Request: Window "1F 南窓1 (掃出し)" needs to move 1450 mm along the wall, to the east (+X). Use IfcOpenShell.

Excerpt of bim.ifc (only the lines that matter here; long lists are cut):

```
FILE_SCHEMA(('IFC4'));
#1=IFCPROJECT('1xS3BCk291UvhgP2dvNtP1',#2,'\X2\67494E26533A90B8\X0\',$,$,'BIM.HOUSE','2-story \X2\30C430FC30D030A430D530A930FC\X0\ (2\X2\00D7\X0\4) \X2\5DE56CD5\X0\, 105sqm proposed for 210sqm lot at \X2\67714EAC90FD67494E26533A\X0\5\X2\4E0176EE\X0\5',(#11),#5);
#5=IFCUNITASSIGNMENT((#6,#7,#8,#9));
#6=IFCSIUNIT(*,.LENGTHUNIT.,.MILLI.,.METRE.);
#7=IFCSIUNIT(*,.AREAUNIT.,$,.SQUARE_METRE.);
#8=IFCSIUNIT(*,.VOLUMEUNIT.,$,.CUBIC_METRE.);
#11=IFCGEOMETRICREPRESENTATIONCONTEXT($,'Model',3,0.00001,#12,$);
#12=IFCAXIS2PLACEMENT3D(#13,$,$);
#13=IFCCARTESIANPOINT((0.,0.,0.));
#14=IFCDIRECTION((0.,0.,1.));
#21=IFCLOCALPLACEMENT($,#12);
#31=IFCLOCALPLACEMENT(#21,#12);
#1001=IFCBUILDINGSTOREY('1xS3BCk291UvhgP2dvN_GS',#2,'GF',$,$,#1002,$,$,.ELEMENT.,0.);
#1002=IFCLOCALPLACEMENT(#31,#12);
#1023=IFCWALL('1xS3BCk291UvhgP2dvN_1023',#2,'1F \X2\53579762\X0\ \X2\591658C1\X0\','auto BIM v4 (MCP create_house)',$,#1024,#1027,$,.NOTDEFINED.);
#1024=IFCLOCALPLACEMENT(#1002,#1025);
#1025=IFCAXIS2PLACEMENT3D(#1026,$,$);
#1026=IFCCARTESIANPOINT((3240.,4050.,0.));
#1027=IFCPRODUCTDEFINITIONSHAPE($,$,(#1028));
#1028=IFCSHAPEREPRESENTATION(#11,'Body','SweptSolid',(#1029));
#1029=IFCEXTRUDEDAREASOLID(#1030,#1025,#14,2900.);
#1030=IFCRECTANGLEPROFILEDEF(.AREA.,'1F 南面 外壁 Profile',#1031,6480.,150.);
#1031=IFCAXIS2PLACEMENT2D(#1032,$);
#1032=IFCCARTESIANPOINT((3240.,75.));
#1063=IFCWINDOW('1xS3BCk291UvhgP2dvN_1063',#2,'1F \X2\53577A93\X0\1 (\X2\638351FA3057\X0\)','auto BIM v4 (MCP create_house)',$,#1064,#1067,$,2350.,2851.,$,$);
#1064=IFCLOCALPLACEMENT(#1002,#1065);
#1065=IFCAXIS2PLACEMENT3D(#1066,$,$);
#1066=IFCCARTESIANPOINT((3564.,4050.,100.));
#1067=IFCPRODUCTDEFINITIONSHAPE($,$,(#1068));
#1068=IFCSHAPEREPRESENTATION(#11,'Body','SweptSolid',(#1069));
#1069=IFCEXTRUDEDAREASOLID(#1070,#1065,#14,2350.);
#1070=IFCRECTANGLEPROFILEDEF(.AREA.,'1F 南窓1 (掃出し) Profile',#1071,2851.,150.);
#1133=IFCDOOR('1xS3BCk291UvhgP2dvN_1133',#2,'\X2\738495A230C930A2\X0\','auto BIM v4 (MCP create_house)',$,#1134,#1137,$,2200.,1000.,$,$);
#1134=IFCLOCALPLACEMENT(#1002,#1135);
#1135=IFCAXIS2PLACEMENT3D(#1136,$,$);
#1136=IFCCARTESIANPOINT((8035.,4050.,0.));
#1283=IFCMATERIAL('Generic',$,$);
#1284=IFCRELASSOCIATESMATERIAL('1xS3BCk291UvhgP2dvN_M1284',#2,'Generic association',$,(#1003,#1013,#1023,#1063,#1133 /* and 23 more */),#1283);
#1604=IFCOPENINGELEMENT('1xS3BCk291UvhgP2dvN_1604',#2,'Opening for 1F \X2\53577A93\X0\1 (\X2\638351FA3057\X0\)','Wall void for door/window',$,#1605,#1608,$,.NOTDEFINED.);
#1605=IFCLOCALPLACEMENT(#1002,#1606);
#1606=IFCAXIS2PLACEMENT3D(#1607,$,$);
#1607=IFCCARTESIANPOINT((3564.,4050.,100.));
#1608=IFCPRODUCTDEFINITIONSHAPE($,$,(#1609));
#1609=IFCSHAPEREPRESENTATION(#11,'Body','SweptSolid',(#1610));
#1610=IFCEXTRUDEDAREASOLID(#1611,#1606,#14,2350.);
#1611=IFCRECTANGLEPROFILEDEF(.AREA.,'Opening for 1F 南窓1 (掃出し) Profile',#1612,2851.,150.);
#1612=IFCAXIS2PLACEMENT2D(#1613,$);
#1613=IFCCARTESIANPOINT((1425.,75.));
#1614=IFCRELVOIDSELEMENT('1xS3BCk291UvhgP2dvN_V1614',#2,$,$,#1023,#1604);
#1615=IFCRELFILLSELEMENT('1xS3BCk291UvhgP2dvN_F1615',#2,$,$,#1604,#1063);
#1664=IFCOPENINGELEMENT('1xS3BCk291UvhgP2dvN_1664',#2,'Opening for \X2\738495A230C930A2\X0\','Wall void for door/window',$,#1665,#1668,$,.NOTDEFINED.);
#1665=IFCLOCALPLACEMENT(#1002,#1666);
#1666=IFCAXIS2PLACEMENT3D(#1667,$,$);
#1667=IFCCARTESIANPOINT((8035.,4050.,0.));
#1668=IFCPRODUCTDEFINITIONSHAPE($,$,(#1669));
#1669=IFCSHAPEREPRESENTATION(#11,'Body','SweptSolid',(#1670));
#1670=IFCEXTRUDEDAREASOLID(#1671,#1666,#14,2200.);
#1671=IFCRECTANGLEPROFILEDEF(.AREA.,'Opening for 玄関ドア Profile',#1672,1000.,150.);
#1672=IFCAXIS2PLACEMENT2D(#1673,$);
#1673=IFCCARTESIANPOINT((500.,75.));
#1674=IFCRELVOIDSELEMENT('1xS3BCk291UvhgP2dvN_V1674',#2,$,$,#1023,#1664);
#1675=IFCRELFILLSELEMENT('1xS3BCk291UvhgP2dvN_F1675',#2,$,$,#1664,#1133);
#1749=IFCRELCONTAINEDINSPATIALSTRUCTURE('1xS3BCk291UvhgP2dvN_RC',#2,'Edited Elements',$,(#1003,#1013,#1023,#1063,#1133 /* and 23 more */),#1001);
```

```python
import ifcopenshell
import ifcopenshell.api.geometry
import ifcopenshell.util.placement
import ifcopenshell.util.unit

model = ifcopenshell.open("bim.ifc")
unit_scale = ifcopenshell.util.unit.calculate_unit_scale(model)

window = model.by_guid("1xS3BCk291UvhgP2dvN_1063")
opening = window.FillsVoids[0].RelatingOpeningElement
wall = opening.VoidsElements[0].RelatingBuildingElement

wall_matrix = ifcopenshell.util.placement.get_local_placement(wall.ObjectPlacement)
shift = wall_matrix[:3, 0] * 1.45 / unit_scale
before = ifcopenshell.util.placement.get_local_placement(window.ObjectPlacement)[:3, 3].copy()

# The window is not placed relative to its opening, so move both.
for product in (opening, window):
    matrix = ifcopenshell.util.placement.get_local_placement(product.ObjectPlacement)
    matrix[:3, 3] += shift
    ifcopenshell.api.geometry.edit_object_placement(model, product=product, matrix=matrix, is_si=False)

after = ifcopenshell.util.placement.get_local_placement(window.ObjectPlacement)[:3, 3]
print("window moved by", (after - before).round(3) + 0.0)

model.write("bim_edited.ifc")
```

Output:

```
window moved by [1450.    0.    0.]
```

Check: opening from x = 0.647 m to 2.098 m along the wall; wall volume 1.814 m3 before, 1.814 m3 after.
